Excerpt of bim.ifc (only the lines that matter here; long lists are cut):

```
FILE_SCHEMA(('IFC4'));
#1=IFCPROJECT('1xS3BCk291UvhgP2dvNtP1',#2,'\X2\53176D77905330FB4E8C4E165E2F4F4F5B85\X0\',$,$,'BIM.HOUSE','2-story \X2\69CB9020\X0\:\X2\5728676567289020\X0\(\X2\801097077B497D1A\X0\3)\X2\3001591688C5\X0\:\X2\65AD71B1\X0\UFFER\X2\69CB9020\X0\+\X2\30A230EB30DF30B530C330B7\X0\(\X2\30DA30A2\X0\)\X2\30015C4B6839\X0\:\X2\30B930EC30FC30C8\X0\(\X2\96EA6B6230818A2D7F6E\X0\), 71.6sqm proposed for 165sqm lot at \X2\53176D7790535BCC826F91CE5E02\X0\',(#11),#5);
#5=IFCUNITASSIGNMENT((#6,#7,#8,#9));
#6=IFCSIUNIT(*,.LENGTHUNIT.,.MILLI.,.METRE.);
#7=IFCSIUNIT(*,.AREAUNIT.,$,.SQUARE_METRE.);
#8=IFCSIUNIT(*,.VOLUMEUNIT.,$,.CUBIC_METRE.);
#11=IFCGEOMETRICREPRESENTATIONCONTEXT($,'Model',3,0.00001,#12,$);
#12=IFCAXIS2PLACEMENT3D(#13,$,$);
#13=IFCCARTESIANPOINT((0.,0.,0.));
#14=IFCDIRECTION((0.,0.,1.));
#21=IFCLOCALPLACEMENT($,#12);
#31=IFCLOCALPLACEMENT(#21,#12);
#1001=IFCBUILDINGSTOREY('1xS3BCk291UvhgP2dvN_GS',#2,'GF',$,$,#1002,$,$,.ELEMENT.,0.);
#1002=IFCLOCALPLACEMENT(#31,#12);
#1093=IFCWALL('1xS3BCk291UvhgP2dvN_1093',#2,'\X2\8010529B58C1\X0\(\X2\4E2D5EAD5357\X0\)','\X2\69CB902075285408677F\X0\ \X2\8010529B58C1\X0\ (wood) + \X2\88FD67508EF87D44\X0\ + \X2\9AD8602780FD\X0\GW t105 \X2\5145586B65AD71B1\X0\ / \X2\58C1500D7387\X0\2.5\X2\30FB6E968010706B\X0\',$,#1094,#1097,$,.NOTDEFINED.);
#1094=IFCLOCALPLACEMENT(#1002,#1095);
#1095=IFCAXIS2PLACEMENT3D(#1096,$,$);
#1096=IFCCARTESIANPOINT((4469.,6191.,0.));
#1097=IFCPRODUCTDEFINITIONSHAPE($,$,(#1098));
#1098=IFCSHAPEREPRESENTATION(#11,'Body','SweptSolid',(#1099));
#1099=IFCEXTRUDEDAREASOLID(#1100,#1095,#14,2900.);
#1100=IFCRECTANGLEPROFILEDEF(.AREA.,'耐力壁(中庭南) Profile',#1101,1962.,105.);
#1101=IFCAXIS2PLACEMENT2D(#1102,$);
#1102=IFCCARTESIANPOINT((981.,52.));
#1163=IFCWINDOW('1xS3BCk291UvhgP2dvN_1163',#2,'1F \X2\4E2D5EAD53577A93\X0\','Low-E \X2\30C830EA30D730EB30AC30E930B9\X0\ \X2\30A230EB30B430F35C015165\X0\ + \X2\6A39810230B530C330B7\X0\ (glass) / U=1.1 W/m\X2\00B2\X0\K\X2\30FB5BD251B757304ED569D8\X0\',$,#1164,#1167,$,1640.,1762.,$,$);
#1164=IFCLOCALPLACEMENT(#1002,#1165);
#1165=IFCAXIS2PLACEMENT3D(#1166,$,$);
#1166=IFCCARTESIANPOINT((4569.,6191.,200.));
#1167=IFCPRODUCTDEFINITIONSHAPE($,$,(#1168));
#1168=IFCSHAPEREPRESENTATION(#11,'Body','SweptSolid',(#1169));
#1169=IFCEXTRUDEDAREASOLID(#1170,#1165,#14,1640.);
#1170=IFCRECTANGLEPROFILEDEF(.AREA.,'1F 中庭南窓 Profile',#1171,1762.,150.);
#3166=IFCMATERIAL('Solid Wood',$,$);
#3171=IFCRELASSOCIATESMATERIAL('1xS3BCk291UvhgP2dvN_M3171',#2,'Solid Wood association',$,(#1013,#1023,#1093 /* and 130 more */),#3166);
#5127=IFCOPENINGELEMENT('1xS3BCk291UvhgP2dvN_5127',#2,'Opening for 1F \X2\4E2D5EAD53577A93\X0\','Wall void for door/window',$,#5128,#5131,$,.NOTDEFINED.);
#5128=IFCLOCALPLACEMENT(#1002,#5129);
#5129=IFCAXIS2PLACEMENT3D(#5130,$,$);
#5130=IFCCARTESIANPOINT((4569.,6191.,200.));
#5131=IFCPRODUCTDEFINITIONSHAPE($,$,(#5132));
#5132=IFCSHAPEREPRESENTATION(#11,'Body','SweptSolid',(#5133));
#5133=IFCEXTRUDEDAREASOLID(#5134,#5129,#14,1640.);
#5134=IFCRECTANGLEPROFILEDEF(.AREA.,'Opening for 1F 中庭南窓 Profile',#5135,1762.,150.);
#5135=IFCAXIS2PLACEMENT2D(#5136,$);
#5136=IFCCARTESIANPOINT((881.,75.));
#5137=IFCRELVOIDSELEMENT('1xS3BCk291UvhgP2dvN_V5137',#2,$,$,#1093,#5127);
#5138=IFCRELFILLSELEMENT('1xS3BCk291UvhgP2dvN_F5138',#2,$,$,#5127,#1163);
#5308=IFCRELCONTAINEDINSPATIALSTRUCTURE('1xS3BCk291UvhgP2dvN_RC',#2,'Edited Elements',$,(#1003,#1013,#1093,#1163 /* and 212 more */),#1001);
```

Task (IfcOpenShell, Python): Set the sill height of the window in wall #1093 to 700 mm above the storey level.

```python
import numpy as np
import ifcopenshell
import ifcopenshell.api.geometry
import ifcopenshell.geom
import ifcopenshell.util.element
import ifcopenshell.util.placement
import ifcopenshell.util.shape
import ifcopenshell.util.unit

model = ifcopenshell.open("bim.ifc")
unit_scale = ifcopenshell.util.unit.calculate_unit_scale(model)

window = model.by_guid("1xS3BCk291UvhgP2dvN_1163")
opening = window.FillsVoids[0].RelatingOpeningElement
storey = ifcopenshell.util.element.get_container(window, ifc_class="IfcBuildingStorey")
level = ifcopenshell.util.placement.get_local_placement(storey.ObjectPlacement)[2, 3]

# The opening's origin need not be at the sill, so measure its lowest point.
shape = ifcopenshell.geom.create_shape(ifcopenshell.geom.settings(), opening)
bottom = ifcopenshell.util.shape.get_shape_bottom_elevation(shape, shape.geometry) / unit_scale
dz = level + 0.7 / unit_scale - bottom

shift = np.array([0.0, 0.0, dz])
# The window is not placed relative to its opening, so move both.
for product in (opening, window):
    matrix = ifcopenshell.util.placement.get_local_placement(product.ObjectPlacement)
    matrix[:3, 3] += shift
    ifcopenshell.api.geometry.edit_object_placement(model, product=product, matrix=matrix, is_si=False)

print(f"moved by {dz * unit_scale:+.3f} m")

model.write("bim_updated.ifc")
```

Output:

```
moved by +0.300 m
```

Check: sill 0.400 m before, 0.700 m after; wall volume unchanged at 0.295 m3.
